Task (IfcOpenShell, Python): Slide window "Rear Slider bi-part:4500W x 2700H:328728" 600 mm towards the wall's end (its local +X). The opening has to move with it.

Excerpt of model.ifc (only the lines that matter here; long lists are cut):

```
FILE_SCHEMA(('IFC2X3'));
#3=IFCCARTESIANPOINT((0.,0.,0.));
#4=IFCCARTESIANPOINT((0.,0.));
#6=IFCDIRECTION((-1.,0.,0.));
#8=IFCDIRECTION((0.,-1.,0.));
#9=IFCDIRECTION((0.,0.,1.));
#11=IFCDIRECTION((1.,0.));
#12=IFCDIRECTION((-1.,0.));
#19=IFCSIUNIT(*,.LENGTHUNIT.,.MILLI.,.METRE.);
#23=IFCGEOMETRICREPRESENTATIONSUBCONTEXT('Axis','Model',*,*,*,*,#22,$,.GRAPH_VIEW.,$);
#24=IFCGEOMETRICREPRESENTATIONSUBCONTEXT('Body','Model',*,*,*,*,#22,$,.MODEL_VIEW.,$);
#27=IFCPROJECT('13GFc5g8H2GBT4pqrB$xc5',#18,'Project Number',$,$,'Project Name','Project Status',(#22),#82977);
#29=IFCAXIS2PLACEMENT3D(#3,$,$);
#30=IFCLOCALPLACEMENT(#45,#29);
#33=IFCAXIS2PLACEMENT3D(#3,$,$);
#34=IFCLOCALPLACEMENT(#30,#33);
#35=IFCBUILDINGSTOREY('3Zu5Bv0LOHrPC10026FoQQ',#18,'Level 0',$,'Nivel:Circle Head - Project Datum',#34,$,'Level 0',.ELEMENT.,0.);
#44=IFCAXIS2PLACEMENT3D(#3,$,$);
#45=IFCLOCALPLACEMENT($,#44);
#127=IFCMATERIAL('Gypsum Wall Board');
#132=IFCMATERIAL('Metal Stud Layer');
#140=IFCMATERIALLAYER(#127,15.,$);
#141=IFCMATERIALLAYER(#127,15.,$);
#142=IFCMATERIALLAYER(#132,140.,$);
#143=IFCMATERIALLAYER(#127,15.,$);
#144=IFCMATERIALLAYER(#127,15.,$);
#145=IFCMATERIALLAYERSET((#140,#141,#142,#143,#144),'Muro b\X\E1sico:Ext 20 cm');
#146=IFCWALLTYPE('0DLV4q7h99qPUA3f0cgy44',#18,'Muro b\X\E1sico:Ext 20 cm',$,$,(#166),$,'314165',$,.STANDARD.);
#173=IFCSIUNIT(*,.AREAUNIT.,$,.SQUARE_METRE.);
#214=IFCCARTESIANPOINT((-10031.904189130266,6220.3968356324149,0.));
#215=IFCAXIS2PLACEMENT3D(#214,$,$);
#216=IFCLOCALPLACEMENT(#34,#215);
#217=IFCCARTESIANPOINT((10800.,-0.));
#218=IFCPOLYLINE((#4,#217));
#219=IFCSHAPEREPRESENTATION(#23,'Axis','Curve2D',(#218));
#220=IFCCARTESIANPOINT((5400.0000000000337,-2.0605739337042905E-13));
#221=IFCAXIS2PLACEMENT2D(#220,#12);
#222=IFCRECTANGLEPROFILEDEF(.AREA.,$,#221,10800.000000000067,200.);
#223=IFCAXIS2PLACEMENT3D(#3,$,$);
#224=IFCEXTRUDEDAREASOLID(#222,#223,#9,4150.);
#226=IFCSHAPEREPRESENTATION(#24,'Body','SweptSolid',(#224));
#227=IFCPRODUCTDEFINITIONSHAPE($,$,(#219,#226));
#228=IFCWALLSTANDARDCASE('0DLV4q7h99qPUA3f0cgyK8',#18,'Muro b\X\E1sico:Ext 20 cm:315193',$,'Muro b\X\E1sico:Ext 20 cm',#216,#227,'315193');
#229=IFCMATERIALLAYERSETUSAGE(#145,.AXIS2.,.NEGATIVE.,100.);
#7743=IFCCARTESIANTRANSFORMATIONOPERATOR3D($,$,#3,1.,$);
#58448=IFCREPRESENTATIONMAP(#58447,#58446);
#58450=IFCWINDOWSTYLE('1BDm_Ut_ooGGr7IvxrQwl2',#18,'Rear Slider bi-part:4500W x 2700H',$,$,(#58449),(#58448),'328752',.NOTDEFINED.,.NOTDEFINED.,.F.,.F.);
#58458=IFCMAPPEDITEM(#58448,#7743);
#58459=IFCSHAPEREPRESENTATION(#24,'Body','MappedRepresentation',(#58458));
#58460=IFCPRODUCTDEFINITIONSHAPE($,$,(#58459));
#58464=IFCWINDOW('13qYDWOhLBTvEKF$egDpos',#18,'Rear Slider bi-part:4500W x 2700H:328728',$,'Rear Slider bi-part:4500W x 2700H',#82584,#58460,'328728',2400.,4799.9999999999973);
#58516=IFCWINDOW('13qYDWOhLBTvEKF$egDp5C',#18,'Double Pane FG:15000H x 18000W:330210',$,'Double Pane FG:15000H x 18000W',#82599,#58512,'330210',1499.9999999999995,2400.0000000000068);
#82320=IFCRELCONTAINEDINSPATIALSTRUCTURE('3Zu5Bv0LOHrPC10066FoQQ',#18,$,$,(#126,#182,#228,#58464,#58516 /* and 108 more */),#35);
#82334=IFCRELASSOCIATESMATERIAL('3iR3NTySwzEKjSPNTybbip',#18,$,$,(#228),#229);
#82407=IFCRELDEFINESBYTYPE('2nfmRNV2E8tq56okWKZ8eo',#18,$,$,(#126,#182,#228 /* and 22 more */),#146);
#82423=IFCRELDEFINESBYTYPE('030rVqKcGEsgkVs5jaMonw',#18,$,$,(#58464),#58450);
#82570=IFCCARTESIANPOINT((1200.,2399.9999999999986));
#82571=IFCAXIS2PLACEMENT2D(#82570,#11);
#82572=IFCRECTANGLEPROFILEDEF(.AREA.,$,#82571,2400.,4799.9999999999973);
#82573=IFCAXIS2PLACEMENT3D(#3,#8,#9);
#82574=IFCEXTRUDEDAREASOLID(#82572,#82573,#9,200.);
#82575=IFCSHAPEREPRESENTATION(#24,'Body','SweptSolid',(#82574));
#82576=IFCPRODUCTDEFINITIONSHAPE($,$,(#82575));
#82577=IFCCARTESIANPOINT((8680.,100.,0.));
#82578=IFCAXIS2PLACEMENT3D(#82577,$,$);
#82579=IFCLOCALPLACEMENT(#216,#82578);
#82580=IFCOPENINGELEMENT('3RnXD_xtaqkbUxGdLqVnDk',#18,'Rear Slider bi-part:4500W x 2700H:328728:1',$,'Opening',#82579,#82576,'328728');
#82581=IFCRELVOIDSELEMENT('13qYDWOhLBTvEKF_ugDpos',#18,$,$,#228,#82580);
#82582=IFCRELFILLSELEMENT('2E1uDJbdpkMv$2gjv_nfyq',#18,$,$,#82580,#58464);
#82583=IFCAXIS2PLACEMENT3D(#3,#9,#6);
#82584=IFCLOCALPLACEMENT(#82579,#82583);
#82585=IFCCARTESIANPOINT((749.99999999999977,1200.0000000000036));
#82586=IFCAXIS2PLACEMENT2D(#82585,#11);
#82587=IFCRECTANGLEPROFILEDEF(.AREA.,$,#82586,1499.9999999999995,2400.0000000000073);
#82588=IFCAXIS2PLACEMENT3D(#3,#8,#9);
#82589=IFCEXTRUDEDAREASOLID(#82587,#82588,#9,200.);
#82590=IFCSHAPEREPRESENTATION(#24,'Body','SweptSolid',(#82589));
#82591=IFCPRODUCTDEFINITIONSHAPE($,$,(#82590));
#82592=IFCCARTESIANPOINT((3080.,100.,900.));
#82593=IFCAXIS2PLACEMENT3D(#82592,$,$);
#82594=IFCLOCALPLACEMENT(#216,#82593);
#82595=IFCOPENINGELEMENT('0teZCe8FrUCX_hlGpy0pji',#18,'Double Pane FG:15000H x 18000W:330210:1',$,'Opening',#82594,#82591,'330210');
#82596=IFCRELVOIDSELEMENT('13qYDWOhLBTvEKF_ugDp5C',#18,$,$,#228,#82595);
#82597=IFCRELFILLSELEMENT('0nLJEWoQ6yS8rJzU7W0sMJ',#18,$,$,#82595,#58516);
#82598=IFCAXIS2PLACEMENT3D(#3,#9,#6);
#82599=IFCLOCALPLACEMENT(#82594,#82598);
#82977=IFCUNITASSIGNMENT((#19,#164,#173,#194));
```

```python
import ifcopenshell
import ifcopenshell.api.geometry
import ifcopenshell.util.placement
import ifcopenshell.util.unit

model = ifcopenshell.open("model.ifc")
unit_scale = ifcopenshell.util.unit.calculate_unit_scale(model)

window = model.by_guid("13qYDWOhLBTvEKF$egDpos")
opening = window.FillsVoids[0].RelatingOpeningElement
wall = opening.VoidsElements[0].RelatingBuildingElement

wall_matrix = ifcopenshell.util.placement.get_local_placement(wall.ObjectPlacement)
shift = wall_matrix[:3, 0] * 0.6 / unit_scale
before = ifcopenshell.util.placement.get_local_placement(window.ObjectPlacement)[:3, 3].copy()

# The window is placed relative to its opening, so it follows when the opening moves.
matrix = ifcopenshell.util.placement.get_local_placement(opening.ObjectPlacement)
matrix[:3, 3] += shift
ifcopenshell.api.geometry.edit_object_placement(
    model, product=opening, matrix=matrix, is_si=False, should_transform_children=True
)

after = ifcopenshell.util.placement.get_local_placement(window.ObjectPlacement)[:3, 3]
print("window moved by", (after - before).round(3) + 0.0)

model.write("model_rev.ifc")
```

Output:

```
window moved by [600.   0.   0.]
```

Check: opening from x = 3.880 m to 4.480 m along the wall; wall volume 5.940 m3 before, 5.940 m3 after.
